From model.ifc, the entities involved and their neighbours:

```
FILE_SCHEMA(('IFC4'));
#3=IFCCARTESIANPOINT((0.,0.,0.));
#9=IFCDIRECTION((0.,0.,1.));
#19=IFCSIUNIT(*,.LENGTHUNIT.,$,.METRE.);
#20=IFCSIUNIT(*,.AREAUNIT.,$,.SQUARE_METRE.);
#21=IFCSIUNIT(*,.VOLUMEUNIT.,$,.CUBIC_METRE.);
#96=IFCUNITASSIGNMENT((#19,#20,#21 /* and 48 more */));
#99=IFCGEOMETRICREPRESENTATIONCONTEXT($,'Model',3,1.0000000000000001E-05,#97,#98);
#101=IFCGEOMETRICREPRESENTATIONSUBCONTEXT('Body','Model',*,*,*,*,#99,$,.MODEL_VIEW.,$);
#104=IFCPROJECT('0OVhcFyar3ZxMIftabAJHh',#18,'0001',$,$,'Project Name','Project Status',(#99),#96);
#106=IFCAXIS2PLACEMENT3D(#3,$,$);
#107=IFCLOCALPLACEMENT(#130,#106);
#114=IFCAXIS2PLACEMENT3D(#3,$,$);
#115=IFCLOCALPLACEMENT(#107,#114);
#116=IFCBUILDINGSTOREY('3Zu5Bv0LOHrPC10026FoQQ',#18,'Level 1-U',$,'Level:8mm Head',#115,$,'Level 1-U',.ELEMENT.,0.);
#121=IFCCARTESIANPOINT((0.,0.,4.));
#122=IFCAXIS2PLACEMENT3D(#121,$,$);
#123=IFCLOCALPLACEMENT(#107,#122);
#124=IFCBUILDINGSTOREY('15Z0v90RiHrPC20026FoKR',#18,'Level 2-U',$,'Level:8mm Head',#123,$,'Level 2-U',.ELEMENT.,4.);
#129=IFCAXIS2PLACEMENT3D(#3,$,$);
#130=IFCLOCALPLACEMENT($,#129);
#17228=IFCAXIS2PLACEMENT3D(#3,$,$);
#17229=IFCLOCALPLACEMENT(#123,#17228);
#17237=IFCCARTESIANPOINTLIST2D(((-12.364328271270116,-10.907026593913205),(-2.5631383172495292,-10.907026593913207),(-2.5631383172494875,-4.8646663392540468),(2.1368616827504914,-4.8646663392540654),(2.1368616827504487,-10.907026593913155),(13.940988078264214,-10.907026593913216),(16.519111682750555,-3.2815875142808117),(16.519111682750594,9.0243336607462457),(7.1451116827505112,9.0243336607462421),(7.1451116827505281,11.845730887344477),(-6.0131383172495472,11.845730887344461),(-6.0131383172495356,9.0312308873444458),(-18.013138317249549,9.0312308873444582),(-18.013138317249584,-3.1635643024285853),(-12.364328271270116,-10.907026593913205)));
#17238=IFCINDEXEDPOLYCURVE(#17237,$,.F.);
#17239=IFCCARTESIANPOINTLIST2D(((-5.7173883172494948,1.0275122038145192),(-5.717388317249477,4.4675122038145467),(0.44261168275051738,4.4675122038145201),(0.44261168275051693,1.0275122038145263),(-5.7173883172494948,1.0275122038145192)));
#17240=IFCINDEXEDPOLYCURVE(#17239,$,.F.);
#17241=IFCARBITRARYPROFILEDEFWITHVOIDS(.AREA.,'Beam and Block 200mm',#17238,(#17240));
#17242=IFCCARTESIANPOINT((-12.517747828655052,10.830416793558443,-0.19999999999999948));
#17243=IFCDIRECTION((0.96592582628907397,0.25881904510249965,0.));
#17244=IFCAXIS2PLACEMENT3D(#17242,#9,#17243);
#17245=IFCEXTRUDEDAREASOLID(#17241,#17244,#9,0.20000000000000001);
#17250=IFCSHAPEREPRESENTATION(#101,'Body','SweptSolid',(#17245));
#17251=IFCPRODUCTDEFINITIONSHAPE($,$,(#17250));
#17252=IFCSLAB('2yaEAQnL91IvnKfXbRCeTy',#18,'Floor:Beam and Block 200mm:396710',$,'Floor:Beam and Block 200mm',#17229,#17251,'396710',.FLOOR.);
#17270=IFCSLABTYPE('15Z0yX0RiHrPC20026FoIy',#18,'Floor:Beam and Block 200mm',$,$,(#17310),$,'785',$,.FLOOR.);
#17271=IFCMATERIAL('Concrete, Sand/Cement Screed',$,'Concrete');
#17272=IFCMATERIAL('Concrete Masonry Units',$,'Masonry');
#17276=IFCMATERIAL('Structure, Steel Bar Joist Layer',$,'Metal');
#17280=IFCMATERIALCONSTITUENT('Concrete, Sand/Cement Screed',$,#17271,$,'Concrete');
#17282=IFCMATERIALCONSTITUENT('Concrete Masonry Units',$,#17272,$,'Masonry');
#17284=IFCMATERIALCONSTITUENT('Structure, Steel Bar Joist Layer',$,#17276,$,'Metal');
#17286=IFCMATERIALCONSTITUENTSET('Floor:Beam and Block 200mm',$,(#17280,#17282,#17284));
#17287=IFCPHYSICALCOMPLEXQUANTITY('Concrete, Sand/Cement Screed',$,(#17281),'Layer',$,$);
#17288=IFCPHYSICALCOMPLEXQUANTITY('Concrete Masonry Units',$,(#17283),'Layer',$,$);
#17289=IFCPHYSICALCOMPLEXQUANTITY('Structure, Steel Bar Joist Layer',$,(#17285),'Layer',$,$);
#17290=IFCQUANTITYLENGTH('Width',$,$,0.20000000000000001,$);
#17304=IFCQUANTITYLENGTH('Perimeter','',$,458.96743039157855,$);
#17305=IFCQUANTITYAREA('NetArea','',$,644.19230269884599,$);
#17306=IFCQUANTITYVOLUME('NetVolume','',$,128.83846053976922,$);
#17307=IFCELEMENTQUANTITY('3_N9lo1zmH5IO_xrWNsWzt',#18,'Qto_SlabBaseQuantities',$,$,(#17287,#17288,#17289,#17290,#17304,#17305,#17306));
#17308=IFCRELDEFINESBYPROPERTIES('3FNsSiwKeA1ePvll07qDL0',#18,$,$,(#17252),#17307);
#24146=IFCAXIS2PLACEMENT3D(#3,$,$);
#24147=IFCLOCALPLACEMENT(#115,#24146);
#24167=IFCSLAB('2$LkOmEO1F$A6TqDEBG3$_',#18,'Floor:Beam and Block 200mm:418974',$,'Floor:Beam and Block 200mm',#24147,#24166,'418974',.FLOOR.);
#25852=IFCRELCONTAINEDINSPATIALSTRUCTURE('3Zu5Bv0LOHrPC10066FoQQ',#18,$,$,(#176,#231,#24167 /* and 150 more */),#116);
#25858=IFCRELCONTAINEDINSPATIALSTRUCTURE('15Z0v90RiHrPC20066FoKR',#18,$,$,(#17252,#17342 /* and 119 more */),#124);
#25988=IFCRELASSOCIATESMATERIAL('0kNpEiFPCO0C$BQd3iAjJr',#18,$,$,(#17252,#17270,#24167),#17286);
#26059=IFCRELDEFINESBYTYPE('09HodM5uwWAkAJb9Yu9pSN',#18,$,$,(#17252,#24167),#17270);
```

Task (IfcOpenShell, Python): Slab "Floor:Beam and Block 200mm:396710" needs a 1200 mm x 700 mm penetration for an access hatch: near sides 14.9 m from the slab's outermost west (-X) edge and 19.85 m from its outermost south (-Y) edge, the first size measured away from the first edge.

```python
import numpy as np
import ifcopenshell
import ifcopenshell.api.feature
import ifcopenshell.api.geometry
import ifcopenshell.api.pset
import ifcopenshell.api.root
import ifcopenshell.geom
import ifcopenshell.util.element
import ifcopenshell.util.placement
import ifcopenshell.util.representation
import ifcopenshell.util.shape
import ifcopenshell.util.unit

model = ifcopenshell.open("model.ifc")
unit_scale = ifcopenshell.util.unit.calculate_unit_scale(model)
area_scale = ifcopenshell.util.unit.calculate_unit_scale(model, "AREAUNIT")
volume_scale = ifcopenshell.util.unit.calculate_unit_scale(model, "VOLUMEUNIT")
settings = ifcopenshell.geom.settings()


def volume(element):
    """Net volume in cubic metres, openings subtracted."""
    shape = ifcopenshell.geom.create_shape(settings, element)
    return ifcopenshell.util.shape.get_volume(shape.geometry)


slab = model.by_guid("2yaEAQnL91IvnKfXbRCeTy")
before = volume(slab)

# Extent in the slab's own axes, in metres. The edges named are its -X and -Y sides.
slab_shape = ifcopenshell.geom.create_shape(settings, slab)
vertices = ifcopenshell.util.shape.get_vertices(slab_shape.geometry)
x_min, y_min, bottom = vertices.min(axis=0)
top = vertices[:, 2].max()

opening = ifcopenshell.api.root.create_entity(model, ifc_class="IfcOpeningElement", name="Access hatch opening", predefined_type="OPENING")
context = ifcopenshell.util.representation.get_context(model, "Model", "Body", "MODEL_VIEW")
width, depth = 1.2, 0.7
outline = [(0.0, 0.0), (width, 0.0), (width, depth), (0.0, depth), (0.0, 0.0)]
# Overshoot both faces by 50 mm so the cut is clean.
shape = ifcopenshell.api.geometry.add_slab_representation(
    model, context=context, depth=top - bottom + 0.1, polyline=outline
)
ifcopenshell.api.geometry.assign_representation(model, product=opening, representation=shape)

matrix = ifcopenshell.util.placement.get_local_placement(slab.ObjectPlacement)
matrix[:, 3] = matrix @ np.append(np.array([x_min + 14.9, y_min + 19.85, bottom - 0.05]) / unit_scale, 1.0)
ifcopenshell.api.geometry.edit_object_placement(model, product=opening, matrix=matrix, is_si=False)
ifcopenshell.api.feature.add_feature(model, feature=opening, element=slab)

after = volume(slab)

# Update the slab's stored quantities.
qto = model.by_id(ifcopenshell.util.element.get_pset(slab, "Qto_SlabBaseQuantities", should_inherit=False)["id"])
ifcopenshell.api.pset.edit_qto(model, qto=qto, properties={
    "NetArea": after / (top - bottom) / area_scale,
    "NetVolume": after / volume_scale,
})

print(f"slab volume {before:.3f} -> {after:.3f} m3")

model.write("model_v2.ifc")
```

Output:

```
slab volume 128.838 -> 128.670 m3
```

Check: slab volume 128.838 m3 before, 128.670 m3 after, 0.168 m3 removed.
